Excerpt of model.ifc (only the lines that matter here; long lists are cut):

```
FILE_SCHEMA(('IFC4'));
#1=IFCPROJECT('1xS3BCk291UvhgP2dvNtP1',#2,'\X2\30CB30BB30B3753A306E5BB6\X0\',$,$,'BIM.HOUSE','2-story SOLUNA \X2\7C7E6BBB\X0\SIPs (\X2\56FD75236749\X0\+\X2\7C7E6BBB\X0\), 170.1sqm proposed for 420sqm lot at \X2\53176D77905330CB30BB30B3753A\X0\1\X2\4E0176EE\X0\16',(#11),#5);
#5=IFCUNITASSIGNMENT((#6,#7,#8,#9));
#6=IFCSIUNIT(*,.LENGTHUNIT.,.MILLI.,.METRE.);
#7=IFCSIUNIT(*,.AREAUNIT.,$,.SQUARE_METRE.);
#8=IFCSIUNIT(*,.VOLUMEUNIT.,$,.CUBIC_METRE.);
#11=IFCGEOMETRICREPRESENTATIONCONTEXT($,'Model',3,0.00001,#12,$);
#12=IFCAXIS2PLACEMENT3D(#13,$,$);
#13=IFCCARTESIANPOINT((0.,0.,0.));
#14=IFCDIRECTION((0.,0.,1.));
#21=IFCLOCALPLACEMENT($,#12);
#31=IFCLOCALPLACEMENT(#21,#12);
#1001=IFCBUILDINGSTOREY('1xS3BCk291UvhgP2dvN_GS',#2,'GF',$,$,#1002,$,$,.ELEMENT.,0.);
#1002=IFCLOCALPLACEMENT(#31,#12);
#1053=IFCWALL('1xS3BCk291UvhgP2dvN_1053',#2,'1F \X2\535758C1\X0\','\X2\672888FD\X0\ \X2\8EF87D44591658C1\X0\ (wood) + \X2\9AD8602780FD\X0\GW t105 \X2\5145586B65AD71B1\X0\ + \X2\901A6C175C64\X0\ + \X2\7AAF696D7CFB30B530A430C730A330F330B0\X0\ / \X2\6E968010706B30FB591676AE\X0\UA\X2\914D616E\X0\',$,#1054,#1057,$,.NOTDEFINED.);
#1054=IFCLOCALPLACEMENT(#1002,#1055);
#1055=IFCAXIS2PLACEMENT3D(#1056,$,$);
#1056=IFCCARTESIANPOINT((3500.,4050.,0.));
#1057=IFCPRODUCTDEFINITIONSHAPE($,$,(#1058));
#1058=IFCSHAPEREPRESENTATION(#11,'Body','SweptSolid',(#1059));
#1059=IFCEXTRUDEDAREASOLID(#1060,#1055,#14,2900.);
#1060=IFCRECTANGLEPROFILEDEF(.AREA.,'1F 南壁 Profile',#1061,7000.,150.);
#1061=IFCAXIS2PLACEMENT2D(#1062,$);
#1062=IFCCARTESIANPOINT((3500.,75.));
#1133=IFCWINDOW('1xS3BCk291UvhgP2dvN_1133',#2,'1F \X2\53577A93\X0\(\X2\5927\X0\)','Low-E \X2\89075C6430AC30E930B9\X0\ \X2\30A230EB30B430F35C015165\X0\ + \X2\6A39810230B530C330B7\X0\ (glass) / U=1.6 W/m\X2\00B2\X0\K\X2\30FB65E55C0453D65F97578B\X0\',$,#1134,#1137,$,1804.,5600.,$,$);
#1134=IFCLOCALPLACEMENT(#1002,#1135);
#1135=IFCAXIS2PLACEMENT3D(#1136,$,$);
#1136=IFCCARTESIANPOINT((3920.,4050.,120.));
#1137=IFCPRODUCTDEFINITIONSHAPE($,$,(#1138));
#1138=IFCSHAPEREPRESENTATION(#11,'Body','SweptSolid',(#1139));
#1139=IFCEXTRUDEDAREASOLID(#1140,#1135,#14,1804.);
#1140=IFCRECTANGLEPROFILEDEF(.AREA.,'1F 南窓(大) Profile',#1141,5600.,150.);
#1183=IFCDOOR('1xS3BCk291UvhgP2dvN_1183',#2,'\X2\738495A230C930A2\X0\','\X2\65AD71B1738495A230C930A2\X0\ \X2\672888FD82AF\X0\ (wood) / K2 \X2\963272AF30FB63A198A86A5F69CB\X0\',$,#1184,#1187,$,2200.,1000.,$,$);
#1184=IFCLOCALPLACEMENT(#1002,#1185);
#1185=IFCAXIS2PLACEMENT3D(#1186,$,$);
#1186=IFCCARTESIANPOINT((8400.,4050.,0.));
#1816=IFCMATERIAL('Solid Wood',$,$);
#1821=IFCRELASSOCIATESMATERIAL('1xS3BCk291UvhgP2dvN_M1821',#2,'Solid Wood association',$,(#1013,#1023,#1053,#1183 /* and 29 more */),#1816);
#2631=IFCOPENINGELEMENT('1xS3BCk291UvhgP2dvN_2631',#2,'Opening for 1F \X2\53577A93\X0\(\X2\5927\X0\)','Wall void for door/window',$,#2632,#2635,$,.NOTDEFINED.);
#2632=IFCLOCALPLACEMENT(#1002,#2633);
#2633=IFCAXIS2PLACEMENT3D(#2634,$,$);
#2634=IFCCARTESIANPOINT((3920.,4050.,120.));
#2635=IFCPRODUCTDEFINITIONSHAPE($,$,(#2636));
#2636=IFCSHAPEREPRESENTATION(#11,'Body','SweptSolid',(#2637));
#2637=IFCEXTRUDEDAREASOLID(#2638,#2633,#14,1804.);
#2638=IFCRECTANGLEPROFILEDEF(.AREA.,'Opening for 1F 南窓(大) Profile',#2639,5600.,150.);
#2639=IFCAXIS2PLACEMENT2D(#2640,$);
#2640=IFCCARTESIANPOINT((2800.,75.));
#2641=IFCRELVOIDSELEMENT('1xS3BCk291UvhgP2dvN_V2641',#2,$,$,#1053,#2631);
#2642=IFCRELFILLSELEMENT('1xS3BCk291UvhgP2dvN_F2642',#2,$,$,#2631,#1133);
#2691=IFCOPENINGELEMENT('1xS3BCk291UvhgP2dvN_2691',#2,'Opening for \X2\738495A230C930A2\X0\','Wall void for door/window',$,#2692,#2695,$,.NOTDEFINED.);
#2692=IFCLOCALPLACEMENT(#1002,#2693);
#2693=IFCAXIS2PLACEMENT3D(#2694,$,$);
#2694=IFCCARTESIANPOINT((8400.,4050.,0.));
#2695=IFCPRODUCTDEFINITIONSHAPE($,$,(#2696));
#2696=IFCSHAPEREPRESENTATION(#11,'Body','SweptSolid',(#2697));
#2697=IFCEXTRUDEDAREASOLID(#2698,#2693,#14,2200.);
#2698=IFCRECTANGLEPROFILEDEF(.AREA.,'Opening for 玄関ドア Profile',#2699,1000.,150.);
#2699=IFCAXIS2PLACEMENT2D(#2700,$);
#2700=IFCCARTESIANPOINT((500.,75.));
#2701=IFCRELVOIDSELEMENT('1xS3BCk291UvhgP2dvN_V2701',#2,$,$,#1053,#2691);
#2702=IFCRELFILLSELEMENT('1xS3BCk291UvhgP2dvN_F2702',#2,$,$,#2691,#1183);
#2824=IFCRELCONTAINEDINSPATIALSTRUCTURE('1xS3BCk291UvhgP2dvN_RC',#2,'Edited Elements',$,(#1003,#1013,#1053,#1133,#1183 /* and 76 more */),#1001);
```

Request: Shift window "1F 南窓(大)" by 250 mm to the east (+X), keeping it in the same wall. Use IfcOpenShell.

```python
import ifcopenshell
import ifcopenshell.api.geometry
import ifcopenshell.util.placement
import ifcopenshell.util.unit

model = ifcopenshell.open("model.ifc")
unit_scale = ifcopenshell.util.unit.calculate_unit_scale(model)

window = model.by_id(1133)
opening = window.FillsVoids[0].RelatingOpeningElement
wall = opening.VoidsElements[0].RelatingBuildingElement

wall_matrix = ifcopenshell.util.placement.get_local_placement(wall.ObjectPlacement)
shift = wall_matrix[:3, 0] * 0.25 / unit_scale
before = ifcopenshell.util.placement.get_local_placement(window.ObjectPlacement)[:3, 3].copy()

# The window is not placed relative to its opening, so move both.
for product in (opening, window):
    matrix = ifcopenshell.util.placement.get_local_placement(product.ObjectPlacement)
    matrix[:3, 3] += shift
    ifcopenshell.api.geometry.edit_object_placement(model, product=product, matrix=matrix, is_si=False)

after = ifcopenshell.util.placement.get_local_placement(window.ObjectPlacement)[:3, 3]
print("window moved by", (after - before).round(3) + 0.0)

model.write("model_v2.ifc")
```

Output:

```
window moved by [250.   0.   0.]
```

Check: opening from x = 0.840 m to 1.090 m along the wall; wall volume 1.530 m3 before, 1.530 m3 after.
